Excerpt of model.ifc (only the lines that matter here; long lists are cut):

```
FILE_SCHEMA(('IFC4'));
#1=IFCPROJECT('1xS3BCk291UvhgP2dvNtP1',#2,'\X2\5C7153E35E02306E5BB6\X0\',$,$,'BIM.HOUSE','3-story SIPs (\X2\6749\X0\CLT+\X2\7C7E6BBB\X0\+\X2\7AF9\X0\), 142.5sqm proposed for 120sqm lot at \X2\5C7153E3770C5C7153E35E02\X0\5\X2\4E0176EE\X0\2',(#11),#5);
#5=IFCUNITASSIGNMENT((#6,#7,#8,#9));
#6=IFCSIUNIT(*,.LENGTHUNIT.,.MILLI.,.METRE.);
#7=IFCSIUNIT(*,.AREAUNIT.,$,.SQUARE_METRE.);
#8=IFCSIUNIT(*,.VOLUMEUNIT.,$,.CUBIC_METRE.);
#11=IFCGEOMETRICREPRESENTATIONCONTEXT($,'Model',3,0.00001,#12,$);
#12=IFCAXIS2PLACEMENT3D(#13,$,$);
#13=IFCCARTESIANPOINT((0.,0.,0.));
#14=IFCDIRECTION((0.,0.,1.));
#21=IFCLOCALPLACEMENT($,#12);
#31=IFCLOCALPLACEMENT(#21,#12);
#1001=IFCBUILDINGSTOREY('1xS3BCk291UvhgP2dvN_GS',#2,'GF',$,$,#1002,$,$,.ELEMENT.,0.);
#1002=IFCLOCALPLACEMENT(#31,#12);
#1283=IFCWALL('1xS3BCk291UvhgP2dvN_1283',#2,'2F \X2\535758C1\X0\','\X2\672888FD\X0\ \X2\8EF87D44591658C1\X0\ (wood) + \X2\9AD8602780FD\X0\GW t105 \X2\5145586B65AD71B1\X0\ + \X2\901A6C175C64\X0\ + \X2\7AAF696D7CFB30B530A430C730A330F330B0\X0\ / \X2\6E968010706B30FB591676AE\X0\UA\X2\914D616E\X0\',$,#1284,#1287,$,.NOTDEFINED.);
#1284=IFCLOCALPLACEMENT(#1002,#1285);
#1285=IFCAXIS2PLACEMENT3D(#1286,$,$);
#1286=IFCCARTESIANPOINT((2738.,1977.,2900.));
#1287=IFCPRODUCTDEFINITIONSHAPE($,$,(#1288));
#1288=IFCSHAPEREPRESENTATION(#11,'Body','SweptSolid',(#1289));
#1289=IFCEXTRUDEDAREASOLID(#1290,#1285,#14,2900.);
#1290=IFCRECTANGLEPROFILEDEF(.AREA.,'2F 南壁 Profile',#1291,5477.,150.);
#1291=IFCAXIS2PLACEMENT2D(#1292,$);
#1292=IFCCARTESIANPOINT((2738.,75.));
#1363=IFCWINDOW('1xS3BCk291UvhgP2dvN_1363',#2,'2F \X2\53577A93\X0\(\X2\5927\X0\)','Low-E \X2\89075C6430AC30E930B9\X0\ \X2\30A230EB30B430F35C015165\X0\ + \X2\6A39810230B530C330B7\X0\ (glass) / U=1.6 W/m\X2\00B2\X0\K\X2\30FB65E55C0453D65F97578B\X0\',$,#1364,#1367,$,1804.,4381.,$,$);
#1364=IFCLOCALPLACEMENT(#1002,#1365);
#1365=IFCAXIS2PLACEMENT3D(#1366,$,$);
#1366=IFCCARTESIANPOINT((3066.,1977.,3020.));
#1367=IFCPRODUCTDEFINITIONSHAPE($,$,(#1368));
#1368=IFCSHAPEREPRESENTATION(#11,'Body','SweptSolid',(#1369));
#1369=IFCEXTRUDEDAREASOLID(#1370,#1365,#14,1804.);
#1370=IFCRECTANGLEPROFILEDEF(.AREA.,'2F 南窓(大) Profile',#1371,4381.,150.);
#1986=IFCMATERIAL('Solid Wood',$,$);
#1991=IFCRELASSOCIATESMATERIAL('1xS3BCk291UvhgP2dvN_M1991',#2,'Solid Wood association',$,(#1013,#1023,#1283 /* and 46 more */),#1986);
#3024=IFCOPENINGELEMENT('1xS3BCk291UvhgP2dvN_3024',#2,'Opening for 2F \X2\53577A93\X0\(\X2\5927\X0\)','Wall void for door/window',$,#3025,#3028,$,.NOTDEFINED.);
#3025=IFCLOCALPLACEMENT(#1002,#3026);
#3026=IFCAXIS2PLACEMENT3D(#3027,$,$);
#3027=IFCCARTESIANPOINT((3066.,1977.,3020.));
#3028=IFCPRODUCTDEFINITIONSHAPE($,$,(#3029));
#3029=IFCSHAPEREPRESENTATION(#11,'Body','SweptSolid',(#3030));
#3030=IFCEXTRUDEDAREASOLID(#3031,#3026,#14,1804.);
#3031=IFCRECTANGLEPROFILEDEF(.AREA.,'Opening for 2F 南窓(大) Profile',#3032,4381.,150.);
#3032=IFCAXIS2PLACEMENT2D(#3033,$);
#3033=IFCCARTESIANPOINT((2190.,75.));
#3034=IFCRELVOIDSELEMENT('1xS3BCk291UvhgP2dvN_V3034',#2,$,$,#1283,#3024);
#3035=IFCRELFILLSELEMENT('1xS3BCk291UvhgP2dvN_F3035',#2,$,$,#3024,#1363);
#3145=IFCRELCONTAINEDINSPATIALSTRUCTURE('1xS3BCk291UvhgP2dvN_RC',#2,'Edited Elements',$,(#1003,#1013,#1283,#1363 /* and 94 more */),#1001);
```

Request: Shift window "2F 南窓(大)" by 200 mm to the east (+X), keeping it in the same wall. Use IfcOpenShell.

```python
import ifcopenshell
import ifcopenshell.api.geometry
import ifcopenshell.util.placement
import ifcopenshell.util.unit

model = ifcopenshell.open("model.ifc")
unit_scale = ifcopenshell.util.unit.calculate_unit_scale(model)

window = model.by_guid("1xS3BCk291UvhgP2dvN_1363")
opening = window.FillsVoids[0].RelatingOpeningElement
wall = opening.VoidsElements[0].RelatingBuildingElement

wall_matrix = ifcopenshell.util.placement.get_local_placement(wall.ObjectPlacement)
shift = wall_matrix[:3, 0] * 0.2 / unit_scale
before = ifcopenshell.util.placement.get_local_placement(window.ObjectPlacement)[:3, 3].copy()

# The window is not placed relative to its opening, so move both.
for product in (opening, window):
    matrix = ifcopenshell.util.placement.get_local_placement(product.ObjectPlacement)
    matrix[:3, 3] += shift
    ifcopenshell.api.geometry.edit_object_placement(model, product=product, matrix=matrix, is_si=False)

after = ifcopenshell.util.placement.get_local_placement(window.ObjectPlacement)[:3, 3]
print("window moved by", (after - before).round(3) + 0.0)

model.write("model_updated.ifc")
```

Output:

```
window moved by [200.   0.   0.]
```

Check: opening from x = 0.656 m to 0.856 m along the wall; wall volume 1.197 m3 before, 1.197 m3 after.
